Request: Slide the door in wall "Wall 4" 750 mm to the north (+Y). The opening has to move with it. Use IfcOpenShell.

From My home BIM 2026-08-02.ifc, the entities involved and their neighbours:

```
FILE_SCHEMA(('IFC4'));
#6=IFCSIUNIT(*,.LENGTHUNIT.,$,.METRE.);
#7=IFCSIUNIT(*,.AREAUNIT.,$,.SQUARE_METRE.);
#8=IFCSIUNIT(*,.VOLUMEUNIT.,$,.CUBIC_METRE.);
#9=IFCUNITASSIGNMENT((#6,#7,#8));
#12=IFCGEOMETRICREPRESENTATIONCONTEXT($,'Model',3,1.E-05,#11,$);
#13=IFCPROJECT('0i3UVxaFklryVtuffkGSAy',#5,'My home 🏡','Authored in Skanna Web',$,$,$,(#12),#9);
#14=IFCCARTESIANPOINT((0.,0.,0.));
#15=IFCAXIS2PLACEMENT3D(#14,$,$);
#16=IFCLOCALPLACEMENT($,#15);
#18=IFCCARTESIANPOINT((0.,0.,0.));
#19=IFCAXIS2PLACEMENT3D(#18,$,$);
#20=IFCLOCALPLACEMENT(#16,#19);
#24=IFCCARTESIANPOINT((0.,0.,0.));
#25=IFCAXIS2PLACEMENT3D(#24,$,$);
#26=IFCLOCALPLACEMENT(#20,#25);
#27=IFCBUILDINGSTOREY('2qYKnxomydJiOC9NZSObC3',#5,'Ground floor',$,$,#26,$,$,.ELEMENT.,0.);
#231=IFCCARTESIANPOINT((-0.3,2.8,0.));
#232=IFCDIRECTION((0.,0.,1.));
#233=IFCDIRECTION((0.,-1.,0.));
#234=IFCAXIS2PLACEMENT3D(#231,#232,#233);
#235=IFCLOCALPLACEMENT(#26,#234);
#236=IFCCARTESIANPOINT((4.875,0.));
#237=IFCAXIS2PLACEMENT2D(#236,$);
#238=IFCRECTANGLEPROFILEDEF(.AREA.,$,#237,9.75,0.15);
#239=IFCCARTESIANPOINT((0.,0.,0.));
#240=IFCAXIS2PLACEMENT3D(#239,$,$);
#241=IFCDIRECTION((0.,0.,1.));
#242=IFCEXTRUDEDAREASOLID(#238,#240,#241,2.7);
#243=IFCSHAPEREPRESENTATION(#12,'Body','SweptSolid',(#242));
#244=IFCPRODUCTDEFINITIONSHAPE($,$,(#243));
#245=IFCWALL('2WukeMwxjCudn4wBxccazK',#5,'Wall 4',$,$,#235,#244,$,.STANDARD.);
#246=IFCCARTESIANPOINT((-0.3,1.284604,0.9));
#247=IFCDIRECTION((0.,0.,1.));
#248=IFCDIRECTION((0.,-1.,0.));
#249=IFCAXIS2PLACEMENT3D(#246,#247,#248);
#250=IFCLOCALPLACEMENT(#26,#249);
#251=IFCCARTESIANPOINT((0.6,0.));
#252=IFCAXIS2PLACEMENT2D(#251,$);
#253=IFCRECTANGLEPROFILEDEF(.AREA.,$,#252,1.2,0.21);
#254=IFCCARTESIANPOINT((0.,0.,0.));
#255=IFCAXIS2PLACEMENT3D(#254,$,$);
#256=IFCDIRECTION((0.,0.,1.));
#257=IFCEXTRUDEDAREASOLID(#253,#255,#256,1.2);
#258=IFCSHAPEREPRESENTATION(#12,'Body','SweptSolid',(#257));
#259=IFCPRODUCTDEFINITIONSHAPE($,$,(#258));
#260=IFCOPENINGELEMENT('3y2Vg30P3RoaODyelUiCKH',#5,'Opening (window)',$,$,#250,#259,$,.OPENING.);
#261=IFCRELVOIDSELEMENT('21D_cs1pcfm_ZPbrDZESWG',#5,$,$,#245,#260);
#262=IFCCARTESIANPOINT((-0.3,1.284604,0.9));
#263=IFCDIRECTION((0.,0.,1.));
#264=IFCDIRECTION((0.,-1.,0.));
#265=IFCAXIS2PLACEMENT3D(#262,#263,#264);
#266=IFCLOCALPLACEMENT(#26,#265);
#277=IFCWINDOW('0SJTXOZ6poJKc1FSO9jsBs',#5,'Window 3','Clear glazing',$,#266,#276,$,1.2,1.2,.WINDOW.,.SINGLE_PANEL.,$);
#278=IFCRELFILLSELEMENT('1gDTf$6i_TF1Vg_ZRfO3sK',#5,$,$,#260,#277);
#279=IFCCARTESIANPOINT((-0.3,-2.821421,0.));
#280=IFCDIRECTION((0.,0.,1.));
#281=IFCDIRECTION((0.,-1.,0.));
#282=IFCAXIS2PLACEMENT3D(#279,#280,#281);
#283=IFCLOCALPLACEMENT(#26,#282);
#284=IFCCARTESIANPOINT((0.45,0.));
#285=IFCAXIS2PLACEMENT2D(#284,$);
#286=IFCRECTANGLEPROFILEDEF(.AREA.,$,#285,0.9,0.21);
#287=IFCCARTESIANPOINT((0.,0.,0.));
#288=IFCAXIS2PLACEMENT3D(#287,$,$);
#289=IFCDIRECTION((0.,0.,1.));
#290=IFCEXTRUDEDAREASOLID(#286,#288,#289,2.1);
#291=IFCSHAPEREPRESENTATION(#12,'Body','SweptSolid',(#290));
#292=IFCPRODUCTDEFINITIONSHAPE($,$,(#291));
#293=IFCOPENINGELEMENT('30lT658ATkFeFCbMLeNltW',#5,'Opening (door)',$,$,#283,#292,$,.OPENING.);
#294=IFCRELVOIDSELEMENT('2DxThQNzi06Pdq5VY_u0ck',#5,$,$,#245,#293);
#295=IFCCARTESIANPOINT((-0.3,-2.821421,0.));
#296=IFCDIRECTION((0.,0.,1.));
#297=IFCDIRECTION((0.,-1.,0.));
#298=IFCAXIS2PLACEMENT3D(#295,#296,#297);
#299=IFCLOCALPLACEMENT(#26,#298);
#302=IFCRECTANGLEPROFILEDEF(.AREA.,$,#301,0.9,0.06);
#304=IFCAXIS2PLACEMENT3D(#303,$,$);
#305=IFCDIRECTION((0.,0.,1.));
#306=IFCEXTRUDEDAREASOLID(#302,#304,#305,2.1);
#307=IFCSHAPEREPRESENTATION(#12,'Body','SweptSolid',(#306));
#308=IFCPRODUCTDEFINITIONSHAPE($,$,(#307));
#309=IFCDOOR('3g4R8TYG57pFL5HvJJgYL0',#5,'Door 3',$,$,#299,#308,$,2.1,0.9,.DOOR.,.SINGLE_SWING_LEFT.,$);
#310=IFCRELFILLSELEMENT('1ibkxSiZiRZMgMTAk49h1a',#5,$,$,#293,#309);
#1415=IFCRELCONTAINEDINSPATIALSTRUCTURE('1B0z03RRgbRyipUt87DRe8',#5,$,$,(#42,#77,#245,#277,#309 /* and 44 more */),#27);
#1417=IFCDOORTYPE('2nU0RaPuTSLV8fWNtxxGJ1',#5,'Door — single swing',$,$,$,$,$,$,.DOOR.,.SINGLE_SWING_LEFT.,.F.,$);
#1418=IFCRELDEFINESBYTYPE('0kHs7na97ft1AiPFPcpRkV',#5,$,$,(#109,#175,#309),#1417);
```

```python
import ifcopenshell
import ifcopenshell.api.geometry
import ifcopenshell.util.placement
import ifcopenshell.util.unit

model = ifcopenshell.open("My home BIM 2026-08-02.ifc")
unit_scale = ifcopenshell.util.unit.calculate_unit_scale(model)

door = model.by_id(309)
opening = door.FillsVoids[0].RelatingOpeningElement
wall = opening.VoidsElements[0].RelatingBuildingElement

wall_matrix = ifcopenshell.util.placement.get_local_placement(wall.ObjectPlacement)
shift = wall_matrix[:3, 0] * -0.75 / unit_scale
before = ifcopenshell.util.placement.get_local_placement(door.ObjectPlacement)[:3, 3].copy()

# The door is not placed relative to its opening, so move both.
for product in (opening, door):
    matrix = ifcopenshell.util.placement.get_local_placement(product.ObjectPlacement)
    matrix[:3, 3] += shift
    ifcopenshell.api.geometry.edit_object_placement(model, product=product, matrix=matrix, is_si=False)

after = ifcopenshell.util.placement.get_local_placement(door.ObjectPlacement)[:3, 3]
print("door moved by", (after - before).round(3) + 0.0)

model.write("My home BIM 2026-08-02-out.ifc")
```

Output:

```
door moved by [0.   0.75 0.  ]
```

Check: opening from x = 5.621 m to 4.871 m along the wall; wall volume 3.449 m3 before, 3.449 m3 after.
